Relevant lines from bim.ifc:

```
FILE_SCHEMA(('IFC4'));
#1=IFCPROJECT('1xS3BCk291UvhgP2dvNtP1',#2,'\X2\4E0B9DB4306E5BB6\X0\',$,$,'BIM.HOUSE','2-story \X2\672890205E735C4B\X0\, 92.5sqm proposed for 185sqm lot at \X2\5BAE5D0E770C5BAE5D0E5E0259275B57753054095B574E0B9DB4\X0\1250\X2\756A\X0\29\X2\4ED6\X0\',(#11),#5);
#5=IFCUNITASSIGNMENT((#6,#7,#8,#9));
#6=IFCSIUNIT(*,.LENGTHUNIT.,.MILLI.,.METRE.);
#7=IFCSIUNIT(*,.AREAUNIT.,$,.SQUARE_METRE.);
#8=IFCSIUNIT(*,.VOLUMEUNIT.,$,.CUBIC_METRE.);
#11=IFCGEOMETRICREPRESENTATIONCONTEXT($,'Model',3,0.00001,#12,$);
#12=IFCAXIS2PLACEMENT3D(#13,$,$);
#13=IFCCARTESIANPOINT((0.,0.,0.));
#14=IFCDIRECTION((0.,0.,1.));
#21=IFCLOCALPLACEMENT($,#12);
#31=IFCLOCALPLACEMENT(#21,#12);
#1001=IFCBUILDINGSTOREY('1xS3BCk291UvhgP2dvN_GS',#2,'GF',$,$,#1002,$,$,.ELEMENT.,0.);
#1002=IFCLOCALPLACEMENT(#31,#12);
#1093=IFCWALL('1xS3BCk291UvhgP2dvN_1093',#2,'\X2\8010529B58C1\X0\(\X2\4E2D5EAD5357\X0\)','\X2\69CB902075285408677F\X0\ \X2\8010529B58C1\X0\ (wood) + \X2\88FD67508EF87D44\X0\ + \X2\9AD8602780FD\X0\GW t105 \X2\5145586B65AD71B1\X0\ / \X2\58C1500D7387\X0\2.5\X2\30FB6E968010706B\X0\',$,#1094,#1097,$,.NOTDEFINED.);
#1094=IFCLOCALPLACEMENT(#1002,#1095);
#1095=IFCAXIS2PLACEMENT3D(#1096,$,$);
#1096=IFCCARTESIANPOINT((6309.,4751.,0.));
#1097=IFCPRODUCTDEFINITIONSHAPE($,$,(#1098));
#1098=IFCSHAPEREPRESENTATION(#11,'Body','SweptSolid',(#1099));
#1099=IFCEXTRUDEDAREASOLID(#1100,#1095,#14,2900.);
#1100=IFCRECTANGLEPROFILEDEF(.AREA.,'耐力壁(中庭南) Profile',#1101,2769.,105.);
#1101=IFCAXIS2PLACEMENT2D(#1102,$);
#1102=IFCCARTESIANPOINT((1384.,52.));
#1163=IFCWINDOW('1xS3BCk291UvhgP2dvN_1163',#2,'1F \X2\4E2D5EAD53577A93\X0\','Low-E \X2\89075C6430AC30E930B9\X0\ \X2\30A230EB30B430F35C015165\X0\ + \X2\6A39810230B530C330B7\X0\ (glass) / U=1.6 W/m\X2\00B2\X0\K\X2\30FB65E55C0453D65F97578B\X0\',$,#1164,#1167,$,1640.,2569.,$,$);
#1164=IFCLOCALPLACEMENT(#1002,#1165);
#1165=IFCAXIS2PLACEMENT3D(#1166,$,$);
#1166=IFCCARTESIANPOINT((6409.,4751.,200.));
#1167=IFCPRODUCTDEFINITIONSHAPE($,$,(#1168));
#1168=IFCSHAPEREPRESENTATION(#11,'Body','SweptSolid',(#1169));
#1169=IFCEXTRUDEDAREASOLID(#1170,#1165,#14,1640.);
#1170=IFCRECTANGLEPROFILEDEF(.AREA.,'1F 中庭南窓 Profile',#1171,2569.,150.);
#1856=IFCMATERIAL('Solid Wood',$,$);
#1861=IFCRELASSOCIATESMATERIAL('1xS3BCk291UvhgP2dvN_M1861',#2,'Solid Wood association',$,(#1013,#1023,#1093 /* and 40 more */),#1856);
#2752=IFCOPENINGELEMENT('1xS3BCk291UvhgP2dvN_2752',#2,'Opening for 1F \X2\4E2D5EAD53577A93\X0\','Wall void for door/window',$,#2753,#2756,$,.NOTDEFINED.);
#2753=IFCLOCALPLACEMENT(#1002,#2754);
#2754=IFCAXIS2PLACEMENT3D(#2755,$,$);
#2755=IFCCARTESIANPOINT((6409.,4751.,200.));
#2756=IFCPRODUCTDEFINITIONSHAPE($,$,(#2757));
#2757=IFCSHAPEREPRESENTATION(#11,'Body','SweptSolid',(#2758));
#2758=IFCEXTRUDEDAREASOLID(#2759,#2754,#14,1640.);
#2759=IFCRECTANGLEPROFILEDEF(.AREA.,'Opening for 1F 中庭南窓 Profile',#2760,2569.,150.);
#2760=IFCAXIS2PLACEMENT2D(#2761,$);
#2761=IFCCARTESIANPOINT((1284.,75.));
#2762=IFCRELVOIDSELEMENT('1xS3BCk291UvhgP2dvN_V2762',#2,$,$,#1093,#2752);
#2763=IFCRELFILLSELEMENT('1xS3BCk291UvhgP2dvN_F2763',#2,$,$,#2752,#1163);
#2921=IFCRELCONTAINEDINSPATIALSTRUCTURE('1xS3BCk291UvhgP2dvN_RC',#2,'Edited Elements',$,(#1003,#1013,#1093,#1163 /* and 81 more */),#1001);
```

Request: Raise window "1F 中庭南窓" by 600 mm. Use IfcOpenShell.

```python
import numpy as np
import ifcopenshell
import ifcopenshell.api.geometry
import ifcopenshell.util.placement
import ifcopenshell.util.unit

model = ifcopenshell.open("bim.ifc")
unit_scale = ifcopenshell.util.unit.calculate_unit_scale(model)

window = model.by_guid("1xS3BCk291UvhgP2dvN_1163")
opening = window.FillsVoids[0].RelatingOpeningElement
dz = 0.6 / unit_scale

shift = np.array([0.0, 0.0, dz])
# The window is not placed relative to its opening, so move both.
for product in (opening, window):
    matrix = ifcopenshell.util.placement.get_local_placement(product.ObjectPlacement)
    matrix[:3, 3] += shift
    ifcopenshell.api.geometry.edit_object_placement(model, product=product, matrix=matrix, is_si=False)

print(f"moved by {dz * unit_scale:+.3f} m")

model.write("bim_v2.ifc")
```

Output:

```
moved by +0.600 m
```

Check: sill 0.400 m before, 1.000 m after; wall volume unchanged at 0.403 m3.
